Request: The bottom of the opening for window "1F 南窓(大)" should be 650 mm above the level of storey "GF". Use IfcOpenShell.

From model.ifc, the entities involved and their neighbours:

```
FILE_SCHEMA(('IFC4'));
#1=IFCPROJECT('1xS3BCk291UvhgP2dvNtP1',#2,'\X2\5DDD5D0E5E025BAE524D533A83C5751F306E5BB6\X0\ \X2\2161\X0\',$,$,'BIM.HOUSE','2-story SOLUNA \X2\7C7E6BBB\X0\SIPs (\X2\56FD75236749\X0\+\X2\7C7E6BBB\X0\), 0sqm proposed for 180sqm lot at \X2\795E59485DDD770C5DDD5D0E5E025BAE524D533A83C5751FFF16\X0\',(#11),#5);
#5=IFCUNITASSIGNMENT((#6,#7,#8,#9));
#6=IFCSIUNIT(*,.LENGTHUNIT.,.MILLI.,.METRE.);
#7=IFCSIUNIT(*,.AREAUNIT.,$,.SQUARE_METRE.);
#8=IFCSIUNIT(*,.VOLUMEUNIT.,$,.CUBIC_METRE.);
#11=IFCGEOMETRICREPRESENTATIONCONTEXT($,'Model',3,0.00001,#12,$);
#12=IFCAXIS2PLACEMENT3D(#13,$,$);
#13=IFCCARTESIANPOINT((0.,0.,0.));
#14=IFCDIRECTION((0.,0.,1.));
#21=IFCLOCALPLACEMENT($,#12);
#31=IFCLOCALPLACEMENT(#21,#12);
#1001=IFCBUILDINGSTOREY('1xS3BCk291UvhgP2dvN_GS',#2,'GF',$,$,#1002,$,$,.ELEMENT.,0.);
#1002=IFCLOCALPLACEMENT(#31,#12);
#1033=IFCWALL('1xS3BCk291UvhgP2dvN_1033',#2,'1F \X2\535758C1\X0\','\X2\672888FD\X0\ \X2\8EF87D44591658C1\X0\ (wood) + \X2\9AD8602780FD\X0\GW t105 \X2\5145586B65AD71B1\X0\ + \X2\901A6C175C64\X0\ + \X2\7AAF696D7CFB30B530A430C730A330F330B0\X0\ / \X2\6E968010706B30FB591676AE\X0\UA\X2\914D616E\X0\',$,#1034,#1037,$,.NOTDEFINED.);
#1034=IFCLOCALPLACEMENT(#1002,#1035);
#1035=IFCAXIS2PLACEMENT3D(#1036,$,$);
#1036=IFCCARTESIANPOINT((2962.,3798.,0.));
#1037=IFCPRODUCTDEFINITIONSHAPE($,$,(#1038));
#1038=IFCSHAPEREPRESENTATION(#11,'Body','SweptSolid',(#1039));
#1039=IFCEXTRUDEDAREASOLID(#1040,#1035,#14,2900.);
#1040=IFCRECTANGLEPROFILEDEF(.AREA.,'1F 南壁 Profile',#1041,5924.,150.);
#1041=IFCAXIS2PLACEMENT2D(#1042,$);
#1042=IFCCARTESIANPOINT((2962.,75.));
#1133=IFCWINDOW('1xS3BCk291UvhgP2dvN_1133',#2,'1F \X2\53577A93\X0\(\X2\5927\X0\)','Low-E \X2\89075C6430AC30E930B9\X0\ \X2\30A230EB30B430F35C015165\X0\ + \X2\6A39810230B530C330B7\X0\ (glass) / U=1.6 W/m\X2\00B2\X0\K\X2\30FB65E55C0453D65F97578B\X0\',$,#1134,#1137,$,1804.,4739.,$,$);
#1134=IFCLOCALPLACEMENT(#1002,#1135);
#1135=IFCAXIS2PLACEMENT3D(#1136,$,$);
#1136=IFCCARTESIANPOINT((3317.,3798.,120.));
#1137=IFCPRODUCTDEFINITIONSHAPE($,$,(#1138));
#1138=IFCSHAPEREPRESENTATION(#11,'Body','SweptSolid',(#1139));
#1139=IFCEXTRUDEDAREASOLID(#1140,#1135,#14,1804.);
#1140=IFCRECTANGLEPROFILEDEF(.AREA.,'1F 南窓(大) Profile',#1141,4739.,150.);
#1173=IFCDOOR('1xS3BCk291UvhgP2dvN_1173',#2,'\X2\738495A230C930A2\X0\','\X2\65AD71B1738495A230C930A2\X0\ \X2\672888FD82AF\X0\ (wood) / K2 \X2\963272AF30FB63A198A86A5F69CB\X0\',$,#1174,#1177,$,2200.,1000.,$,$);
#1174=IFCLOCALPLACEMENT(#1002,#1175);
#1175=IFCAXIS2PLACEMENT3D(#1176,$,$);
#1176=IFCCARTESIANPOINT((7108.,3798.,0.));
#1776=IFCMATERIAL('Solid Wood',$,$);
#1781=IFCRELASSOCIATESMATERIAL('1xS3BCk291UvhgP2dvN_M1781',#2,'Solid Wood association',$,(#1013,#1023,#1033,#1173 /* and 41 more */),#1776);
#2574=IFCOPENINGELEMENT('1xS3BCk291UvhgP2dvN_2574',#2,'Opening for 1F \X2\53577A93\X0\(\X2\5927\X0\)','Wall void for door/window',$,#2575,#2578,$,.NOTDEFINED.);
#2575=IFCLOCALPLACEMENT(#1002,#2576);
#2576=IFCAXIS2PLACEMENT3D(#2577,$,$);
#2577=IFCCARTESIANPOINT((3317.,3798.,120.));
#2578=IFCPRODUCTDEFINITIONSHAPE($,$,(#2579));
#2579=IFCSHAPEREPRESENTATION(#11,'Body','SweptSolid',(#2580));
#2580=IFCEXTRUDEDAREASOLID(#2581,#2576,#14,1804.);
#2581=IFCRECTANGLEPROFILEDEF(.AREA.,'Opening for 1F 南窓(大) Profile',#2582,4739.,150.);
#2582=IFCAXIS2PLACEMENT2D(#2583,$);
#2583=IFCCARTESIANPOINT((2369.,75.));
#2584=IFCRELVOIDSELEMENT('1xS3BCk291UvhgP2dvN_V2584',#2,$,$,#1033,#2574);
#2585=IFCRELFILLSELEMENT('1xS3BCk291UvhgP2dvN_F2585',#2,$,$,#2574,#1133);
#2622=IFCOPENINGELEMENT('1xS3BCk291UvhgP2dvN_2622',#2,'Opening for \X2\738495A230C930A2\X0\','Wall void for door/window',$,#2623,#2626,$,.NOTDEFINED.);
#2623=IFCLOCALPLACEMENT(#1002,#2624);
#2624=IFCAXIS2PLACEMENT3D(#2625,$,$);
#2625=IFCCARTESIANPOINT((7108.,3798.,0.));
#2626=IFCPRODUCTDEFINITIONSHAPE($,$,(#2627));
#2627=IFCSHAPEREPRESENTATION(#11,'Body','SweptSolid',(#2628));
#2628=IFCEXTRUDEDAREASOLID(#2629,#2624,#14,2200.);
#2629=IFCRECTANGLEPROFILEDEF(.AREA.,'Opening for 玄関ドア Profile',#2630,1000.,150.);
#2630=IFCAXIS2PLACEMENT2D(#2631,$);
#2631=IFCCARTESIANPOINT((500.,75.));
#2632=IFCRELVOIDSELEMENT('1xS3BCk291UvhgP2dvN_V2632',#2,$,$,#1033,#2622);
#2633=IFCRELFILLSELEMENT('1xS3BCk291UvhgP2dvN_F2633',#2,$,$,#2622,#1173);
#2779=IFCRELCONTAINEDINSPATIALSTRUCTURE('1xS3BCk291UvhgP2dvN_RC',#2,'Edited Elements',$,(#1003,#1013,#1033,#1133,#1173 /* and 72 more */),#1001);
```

```python
import numpy as np
import ifcopenshell
import ifcopenshell.api.geometry
import ifcopenshell.geom
import ifcopenshell.util.element
import ifcopenshell.util.placement
import ifcopenshell.util.shape
import ifcopenshell.util.unit

model = ifcopenshell.open("model.ifc")
unit_scale = ifcopenshell.util.unit.calculate_unit_scale(model)

window = model.by_id(1133)
opening = window.FillsVoids[0].RelatingOpeningElement
storey = ifcopenshell.util.element.get_container(window, ifc_class="IfcBuildingStorey")
level = ifcopenshell.util.placement.get_local_placement(storey.ObjectPlacement)[2, 3]

# The opening's origin need not be at the sill, so measure its lowest point.
shape = ifcopenshell.geom.create_shape(ifcopenshell.geom.settings(), opening)
bottom = ifcopenshell.util.shape.get_shape_bottom_elevation(shape, shape.geometry) / unit_scale
dz = level + 650.0 - bottom

shift = np.array([0.0, 0.0, dz])
# The window is not placed relative to its opening, so move both.
for product in (opening, window):
    matrix = ifcopenshell.util.placement.get_local_placement(product.ObjectPlacement)
    matrix[:3, 3] += shift
    ifcopenshell.api.geometry.edit_object_placement(model, product=product, matrix=matrix, is_si=False)

print(f"moved by {dz * unit_scale:+.3f} m")

model.write("model_edited.ifc")
```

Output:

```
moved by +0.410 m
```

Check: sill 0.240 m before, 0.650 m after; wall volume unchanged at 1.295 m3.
